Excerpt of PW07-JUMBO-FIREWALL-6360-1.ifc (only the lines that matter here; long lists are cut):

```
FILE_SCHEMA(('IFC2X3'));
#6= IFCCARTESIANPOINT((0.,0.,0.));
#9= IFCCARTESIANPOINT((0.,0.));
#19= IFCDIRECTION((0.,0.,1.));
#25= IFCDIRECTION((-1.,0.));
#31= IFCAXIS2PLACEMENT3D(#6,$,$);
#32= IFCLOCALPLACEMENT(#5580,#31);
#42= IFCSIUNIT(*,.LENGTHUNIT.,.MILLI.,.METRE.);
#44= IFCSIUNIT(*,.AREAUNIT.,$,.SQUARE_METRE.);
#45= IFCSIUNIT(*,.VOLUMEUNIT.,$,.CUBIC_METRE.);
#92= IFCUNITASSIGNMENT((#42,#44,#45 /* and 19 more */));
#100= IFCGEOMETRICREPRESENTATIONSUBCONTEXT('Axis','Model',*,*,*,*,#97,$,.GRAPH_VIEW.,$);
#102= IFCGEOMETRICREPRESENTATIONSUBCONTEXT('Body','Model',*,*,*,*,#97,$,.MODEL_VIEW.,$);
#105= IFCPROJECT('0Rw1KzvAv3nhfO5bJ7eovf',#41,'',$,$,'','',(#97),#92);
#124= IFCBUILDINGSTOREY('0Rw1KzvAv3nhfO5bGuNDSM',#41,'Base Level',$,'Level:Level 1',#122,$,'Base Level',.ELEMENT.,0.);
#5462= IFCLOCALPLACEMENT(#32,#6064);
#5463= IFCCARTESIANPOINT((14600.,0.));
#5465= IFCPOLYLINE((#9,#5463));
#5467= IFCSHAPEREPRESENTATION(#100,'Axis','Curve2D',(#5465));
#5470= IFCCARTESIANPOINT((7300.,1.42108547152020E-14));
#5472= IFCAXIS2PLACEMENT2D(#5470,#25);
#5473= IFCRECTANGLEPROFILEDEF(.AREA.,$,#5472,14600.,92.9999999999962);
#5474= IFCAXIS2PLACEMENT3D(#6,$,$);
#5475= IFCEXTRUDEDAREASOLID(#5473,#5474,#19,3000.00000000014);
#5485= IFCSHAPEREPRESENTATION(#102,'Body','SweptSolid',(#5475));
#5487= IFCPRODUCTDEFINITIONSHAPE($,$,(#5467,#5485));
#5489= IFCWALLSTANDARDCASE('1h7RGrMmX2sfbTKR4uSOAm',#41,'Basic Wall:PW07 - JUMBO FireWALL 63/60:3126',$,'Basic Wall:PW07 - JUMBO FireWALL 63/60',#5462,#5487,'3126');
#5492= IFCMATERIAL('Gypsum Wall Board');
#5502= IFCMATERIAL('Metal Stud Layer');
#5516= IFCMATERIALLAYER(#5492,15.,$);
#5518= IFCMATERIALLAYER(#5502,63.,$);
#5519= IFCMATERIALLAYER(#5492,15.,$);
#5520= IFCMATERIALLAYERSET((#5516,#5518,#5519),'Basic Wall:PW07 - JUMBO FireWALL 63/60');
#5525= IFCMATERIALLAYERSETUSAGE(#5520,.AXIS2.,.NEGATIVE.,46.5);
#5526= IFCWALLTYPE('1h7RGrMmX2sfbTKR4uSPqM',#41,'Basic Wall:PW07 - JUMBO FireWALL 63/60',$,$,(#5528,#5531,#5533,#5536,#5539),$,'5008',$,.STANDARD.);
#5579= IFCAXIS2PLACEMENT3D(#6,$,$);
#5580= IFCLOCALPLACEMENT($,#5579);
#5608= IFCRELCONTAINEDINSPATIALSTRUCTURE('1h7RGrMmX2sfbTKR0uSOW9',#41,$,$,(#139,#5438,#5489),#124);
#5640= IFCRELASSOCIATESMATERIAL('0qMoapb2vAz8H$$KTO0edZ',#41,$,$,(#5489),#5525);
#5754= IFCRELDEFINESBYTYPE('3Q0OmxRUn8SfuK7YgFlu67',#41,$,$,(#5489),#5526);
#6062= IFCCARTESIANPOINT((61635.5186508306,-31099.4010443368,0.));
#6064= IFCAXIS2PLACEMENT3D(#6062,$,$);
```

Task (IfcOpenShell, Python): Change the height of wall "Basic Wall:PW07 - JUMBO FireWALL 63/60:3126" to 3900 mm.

```python
import ifcopenshell
import ifcopenshell.geom
import ifcopenshell.util.representation
import ifcopenshell.util.shape

model = ifcopenshell.open("PW07-JUMBO-FIREWALL-6360-1.ifc")
settings = ifcopenshell.geom.settings()


def volume(element):
    """Net volume in cubic metres, openings subtracted."""
    shape = ifcopenshell.geom.create_shape(settings, element)
    return ifcopenshell.util.shape.get_volume(shape.geometry)


wall = model.by_guid("1h7RGrMmX2sfbTKR4uSOAm")
before = volume(wall)

body = ifcopenshell.util.representation.get_representation(wall, "Model", "Body")
solid = body.Items[0]
old_height = solid.Depth
solid.Depth = 3900.0
after = volume(wall)

print(f"height {old_height:g} -> {solid.Depth:g}, volume {before:.3f} -> {after:.3f} m3")

model.write("PW07-JUMBO-FIREWALL-6360-1_rev.ifc")
```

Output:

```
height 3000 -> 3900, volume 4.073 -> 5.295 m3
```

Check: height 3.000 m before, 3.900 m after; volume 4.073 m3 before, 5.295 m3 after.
